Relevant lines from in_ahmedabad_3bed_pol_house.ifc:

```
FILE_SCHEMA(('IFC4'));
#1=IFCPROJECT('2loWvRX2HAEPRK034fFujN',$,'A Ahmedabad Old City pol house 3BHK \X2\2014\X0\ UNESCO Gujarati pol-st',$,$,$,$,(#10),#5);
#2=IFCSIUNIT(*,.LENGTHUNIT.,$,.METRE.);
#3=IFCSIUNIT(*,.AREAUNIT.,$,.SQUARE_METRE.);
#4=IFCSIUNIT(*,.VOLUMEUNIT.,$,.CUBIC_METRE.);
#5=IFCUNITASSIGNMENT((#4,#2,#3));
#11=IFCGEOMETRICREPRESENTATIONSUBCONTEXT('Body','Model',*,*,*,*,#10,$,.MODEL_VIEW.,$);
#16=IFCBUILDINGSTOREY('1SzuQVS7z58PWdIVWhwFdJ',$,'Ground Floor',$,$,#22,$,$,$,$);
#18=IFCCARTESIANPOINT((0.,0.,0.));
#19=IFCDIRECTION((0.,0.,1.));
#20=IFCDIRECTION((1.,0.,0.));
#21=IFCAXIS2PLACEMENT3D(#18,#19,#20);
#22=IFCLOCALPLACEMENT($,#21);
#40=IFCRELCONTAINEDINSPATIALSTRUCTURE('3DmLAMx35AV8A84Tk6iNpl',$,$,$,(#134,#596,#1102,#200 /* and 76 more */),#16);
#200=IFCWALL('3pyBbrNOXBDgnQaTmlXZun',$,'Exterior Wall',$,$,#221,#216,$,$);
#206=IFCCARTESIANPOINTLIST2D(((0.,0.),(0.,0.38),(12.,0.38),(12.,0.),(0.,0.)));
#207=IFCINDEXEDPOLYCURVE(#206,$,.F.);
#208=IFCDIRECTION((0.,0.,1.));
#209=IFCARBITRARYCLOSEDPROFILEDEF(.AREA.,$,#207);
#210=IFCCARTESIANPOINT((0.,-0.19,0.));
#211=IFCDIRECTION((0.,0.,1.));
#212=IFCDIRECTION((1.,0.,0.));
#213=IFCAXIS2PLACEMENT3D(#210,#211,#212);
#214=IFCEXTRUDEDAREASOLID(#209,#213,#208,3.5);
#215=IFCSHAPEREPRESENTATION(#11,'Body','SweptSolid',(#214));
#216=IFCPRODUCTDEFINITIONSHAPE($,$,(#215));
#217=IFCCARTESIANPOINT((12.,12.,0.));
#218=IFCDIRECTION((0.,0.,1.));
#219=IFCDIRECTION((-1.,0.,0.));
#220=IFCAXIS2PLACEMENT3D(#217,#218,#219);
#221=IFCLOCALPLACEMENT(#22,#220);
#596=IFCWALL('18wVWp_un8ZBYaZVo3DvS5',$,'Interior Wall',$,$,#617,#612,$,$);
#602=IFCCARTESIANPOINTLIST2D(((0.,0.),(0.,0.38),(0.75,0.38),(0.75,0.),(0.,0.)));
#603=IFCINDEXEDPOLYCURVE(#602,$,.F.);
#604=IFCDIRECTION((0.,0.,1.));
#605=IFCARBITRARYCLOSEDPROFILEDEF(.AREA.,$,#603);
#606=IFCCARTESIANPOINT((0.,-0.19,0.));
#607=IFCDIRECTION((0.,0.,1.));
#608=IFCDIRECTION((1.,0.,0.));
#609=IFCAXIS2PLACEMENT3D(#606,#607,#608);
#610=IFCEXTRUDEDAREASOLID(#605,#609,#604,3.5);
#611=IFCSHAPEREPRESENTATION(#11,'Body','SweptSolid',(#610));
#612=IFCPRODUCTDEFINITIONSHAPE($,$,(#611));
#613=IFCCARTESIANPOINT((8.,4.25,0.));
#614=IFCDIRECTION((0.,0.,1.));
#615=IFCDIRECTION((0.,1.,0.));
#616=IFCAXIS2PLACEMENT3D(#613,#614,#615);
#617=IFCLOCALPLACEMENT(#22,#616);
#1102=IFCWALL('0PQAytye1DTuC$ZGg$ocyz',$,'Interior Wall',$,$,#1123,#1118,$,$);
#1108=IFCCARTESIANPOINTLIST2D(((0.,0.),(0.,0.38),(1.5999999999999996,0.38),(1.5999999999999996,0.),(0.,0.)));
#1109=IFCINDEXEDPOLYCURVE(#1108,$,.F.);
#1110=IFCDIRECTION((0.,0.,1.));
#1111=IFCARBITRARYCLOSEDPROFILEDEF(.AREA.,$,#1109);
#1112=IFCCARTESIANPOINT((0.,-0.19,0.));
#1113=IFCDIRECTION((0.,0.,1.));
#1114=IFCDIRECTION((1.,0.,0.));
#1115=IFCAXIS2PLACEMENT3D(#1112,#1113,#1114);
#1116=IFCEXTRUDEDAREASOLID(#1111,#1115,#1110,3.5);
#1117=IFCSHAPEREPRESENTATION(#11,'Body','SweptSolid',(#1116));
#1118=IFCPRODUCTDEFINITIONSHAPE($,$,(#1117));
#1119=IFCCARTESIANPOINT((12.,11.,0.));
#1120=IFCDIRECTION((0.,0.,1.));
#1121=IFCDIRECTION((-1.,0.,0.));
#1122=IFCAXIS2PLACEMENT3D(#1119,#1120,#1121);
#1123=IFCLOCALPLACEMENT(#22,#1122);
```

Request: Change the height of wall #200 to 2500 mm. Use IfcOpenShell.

```python
import ifcopenshell
import ifcopenshell.geom
import ifcopenshell.util.representation
import ifcopenshell.util.shape
import ifcopenshell.util.unit

model = ifcopenshell.open("in_ahmedabad_3bed_pol_house.ifc")
unit_scale = ifcopenshell.util.unit.calculate_unit_scale(model)
settings = ifcopenshell.geom.settings()


def volume(element):
    """Net volume in cubic metres, openings subtracted."""
    shape = ifcopenshell.geom.create_shape(settings, element)
    return ifcopenshell.util.shape.get_volume(shape.geometry)


wall = model.by_guid("3pyBbrNOXBDgnQaTmlXZun")
before = volume(wall)

body = ifcopenshell.util.representation.get_representation(wall, "Model", "Body")
solid = body.Items[0]
old_height = solid.Depth
solid.Depth = 2.5 / unit_scale
after = volume(wall)

print(f"height {old_height:g} -> {solid.Depth:g}, volume {before:.3f} -> {after:.3f} m3")

model.write("in_ahmedabad_3bed_pol_house_edited.ifc")
```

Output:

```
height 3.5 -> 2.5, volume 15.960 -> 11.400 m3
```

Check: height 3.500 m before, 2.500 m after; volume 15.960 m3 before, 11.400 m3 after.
